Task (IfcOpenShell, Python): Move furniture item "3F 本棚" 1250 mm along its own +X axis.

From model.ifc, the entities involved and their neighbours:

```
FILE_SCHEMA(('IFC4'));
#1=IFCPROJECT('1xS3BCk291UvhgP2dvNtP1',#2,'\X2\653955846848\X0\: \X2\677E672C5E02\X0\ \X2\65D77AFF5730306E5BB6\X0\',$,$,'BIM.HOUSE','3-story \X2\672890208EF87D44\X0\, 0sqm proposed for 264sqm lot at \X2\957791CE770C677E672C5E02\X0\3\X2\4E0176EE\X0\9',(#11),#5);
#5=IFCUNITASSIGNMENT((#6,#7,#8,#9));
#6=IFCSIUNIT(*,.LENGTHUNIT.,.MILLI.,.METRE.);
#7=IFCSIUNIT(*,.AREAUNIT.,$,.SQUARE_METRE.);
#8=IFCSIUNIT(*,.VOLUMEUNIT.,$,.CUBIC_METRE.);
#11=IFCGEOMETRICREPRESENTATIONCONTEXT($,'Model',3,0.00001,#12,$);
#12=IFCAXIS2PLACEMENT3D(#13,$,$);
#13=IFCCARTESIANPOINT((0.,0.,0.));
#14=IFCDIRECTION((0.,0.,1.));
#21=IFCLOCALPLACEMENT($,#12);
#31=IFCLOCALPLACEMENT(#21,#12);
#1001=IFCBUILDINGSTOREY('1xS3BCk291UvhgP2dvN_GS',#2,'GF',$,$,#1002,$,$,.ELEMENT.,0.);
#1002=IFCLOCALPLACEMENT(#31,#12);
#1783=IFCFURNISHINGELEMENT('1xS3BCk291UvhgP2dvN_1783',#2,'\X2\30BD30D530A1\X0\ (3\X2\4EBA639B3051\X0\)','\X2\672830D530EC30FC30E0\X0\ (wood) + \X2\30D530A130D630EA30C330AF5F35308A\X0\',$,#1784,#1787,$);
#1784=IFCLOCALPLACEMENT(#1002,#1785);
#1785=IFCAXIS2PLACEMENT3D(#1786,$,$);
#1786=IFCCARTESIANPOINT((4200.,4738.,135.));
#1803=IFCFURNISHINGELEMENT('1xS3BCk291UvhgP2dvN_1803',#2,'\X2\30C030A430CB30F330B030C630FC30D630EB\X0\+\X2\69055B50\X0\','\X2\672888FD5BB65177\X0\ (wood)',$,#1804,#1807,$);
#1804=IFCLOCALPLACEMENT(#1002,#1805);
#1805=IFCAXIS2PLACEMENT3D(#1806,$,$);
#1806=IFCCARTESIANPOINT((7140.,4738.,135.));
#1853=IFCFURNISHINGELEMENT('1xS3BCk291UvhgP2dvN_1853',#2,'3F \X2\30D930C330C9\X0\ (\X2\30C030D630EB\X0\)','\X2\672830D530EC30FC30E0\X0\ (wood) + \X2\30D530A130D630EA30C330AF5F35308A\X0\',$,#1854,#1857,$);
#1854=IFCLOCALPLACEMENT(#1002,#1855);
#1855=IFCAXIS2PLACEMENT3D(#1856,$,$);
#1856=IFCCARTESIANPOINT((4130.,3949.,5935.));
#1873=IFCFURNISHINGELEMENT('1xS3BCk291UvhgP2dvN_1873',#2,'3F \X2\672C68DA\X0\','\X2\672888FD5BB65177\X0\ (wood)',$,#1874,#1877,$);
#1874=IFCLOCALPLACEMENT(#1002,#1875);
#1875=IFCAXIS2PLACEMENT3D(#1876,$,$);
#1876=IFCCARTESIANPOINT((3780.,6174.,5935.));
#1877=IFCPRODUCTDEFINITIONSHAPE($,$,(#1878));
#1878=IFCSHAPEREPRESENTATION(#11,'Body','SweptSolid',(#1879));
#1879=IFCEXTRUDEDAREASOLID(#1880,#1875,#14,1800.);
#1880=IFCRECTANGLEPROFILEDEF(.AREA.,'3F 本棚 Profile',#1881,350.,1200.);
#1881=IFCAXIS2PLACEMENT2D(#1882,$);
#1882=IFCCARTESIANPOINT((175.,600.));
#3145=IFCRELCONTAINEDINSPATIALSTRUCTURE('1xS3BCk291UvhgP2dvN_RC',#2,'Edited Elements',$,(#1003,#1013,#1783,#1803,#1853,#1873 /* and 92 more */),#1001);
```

```python
import ifcopenshell
import ifcopenshell.api.geometry
import ifcopenshell.util.placement
import ifcopenshell.util.unit

model = ifcopenshell.open("model.ifc")
unit_scale = ifcopenshell.util.unit.calculate_unit_scale(model)

item = model.by_id(1873)
matrix = ifcopenshell.util.placement.get_local_placement(item.ObjectPlacement)
matrix[:3, 3] += matrix[:3, 0] * 1.25 / unit_scale
ifcopenshell.api.geometry.edit_object_placement(model, product=item, matrix=matrix, is_si=False)

print(ifcopenshell.util.placement.get_local_placement(item.ObjectPlacement).round(3) + 0.0)

model.write("model_edited.ifc")
```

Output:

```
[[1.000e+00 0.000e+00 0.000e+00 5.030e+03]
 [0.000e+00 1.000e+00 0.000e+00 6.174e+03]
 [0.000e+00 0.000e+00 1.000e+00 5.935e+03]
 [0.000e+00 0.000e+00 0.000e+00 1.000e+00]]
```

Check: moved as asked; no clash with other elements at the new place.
